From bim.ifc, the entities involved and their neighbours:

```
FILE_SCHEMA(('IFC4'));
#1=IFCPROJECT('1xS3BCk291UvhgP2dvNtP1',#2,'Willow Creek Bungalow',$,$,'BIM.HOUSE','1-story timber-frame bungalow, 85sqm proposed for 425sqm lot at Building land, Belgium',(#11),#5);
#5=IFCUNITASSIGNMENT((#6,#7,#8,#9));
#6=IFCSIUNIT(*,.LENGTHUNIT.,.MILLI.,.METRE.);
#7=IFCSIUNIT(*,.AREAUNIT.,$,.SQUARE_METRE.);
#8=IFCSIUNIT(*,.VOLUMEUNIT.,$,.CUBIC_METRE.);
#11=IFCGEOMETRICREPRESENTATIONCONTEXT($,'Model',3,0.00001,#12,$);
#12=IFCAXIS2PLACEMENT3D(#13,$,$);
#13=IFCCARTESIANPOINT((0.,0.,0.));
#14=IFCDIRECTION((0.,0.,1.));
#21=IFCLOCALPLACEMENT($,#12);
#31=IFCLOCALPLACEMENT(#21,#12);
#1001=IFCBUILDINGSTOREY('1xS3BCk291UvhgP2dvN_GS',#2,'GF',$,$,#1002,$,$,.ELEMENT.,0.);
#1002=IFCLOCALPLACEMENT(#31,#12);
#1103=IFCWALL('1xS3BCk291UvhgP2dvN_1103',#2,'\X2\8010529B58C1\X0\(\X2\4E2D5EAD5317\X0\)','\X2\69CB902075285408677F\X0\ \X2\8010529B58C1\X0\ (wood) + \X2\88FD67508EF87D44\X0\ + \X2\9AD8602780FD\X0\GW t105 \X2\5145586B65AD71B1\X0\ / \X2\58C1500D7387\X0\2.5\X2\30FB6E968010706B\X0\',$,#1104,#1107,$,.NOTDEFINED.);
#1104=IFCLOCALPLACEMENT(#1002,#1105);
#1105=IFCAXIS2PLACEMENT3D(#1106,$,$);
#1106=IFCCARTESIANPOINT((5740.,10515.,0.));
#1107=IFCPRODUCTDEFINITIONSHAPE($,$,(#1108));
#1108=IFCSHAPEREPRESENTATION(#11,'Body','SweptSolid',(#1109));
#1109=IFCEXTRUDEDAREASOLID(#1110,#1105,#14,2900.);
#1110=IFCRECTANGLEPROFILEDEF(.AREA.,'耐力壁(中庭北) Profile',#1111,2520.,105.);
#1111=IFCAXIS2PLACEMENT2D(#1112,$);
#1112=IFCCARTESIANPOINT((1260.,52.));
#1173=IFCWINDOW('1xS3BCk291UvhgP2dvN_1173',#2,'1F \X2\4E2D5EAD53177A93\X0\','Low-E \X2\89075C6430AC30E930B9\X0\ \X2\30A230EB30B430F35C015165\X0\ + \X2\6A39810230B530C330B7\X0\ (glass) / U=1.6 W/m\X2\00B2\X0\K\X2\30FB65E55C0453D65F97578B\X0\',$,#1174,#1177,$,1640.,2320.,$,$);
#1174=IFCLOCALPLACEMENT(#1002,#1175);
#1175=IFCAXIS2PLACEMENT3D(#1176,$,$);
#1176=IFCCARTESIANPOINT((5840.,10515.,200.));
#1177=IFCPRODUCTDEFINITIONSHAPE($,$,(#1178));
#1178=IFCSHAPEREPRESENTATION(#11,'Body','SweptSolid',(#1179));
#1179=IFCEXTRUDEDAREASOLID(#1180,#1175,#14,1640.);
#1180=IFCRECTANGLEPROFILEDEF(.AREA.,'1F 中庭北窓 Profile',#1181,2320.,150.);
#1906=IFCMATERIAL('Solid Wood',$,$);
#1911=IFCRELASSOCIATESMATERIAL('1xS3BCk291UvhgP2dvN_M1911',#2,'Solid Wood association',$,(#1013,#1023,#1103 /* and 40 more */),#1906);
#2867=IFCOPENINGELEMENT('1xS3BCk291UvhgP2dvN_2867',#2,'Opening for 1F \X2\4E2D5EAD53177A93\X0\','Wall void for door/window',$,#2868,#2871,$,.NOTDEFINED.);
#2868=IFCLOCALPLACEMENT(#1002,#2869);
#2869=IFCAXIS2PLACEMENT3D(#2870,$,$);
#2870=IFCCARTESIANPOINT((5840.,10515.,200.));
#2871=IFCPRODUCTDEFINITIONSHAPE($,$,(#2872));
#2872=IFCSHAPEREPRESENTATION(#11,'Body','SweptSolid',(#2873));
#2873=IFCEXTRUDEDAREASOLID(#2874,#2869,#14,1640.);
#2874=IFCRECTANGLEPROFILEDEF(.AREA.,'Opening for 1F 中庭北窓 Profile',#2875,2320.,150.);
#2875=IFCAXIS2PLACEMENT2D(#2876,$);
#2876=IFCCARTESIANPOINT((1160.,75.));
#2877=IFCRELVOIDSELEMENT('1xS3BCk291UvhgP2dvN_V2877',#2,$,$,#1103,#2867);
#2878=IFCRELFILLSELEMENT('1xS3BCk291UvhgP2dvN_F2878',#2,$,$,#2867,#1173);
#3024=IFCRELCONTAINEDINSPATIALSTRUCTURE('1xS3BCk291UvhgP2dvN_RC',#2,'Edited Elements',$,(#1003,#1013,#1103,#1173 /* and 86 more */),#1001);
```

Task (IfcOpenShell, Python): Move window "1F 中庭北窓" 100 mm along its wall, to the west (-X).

```python
import ifcopenshell
import ifcopenshell.api.geometry
import ifcopenshell.util.placement

model = ifcopenshell.open("bim.ifc")

window = model.by_guid("1xS3BCk291UvhgP2dvN_1173")
opening = window.FillsVoids[0].RelatingOpeningElement
wall = opening.VoidsElements[0].RelatingBuildingElement

wall_matrix = ifcopenshell.util.placement.get_local_placement(wall.ObjectPlacement)
shift = wall_matrix[:3, 0] * -100.0
before = ifcopenshell.util.placement.get_local_placement(window.ObjectPlacement)[:3, 3].copy()

# The window is not placed relative to its opening, so move both.
for product in (opening, window):
    matrix = ifcopenshell.util.placement.get_local_placement(product.ObjectPlacement)
    matrix[:3, 3] += shift
    ifcopenshell.api.geometry.edit_object_placement(model, product=product, matrix=matrix, is_si=False)

after = ifcopenshell.util.placement.get_local_placement(window.ObjectPlacement)[:3, 3]
print("window moved by", (after - before).round(3) + 0.0)

model.write("bim-out.ifc")
```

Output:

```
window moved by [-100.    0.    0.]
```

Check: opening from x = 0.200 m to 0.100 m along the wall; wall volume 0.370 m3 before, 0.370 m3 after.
